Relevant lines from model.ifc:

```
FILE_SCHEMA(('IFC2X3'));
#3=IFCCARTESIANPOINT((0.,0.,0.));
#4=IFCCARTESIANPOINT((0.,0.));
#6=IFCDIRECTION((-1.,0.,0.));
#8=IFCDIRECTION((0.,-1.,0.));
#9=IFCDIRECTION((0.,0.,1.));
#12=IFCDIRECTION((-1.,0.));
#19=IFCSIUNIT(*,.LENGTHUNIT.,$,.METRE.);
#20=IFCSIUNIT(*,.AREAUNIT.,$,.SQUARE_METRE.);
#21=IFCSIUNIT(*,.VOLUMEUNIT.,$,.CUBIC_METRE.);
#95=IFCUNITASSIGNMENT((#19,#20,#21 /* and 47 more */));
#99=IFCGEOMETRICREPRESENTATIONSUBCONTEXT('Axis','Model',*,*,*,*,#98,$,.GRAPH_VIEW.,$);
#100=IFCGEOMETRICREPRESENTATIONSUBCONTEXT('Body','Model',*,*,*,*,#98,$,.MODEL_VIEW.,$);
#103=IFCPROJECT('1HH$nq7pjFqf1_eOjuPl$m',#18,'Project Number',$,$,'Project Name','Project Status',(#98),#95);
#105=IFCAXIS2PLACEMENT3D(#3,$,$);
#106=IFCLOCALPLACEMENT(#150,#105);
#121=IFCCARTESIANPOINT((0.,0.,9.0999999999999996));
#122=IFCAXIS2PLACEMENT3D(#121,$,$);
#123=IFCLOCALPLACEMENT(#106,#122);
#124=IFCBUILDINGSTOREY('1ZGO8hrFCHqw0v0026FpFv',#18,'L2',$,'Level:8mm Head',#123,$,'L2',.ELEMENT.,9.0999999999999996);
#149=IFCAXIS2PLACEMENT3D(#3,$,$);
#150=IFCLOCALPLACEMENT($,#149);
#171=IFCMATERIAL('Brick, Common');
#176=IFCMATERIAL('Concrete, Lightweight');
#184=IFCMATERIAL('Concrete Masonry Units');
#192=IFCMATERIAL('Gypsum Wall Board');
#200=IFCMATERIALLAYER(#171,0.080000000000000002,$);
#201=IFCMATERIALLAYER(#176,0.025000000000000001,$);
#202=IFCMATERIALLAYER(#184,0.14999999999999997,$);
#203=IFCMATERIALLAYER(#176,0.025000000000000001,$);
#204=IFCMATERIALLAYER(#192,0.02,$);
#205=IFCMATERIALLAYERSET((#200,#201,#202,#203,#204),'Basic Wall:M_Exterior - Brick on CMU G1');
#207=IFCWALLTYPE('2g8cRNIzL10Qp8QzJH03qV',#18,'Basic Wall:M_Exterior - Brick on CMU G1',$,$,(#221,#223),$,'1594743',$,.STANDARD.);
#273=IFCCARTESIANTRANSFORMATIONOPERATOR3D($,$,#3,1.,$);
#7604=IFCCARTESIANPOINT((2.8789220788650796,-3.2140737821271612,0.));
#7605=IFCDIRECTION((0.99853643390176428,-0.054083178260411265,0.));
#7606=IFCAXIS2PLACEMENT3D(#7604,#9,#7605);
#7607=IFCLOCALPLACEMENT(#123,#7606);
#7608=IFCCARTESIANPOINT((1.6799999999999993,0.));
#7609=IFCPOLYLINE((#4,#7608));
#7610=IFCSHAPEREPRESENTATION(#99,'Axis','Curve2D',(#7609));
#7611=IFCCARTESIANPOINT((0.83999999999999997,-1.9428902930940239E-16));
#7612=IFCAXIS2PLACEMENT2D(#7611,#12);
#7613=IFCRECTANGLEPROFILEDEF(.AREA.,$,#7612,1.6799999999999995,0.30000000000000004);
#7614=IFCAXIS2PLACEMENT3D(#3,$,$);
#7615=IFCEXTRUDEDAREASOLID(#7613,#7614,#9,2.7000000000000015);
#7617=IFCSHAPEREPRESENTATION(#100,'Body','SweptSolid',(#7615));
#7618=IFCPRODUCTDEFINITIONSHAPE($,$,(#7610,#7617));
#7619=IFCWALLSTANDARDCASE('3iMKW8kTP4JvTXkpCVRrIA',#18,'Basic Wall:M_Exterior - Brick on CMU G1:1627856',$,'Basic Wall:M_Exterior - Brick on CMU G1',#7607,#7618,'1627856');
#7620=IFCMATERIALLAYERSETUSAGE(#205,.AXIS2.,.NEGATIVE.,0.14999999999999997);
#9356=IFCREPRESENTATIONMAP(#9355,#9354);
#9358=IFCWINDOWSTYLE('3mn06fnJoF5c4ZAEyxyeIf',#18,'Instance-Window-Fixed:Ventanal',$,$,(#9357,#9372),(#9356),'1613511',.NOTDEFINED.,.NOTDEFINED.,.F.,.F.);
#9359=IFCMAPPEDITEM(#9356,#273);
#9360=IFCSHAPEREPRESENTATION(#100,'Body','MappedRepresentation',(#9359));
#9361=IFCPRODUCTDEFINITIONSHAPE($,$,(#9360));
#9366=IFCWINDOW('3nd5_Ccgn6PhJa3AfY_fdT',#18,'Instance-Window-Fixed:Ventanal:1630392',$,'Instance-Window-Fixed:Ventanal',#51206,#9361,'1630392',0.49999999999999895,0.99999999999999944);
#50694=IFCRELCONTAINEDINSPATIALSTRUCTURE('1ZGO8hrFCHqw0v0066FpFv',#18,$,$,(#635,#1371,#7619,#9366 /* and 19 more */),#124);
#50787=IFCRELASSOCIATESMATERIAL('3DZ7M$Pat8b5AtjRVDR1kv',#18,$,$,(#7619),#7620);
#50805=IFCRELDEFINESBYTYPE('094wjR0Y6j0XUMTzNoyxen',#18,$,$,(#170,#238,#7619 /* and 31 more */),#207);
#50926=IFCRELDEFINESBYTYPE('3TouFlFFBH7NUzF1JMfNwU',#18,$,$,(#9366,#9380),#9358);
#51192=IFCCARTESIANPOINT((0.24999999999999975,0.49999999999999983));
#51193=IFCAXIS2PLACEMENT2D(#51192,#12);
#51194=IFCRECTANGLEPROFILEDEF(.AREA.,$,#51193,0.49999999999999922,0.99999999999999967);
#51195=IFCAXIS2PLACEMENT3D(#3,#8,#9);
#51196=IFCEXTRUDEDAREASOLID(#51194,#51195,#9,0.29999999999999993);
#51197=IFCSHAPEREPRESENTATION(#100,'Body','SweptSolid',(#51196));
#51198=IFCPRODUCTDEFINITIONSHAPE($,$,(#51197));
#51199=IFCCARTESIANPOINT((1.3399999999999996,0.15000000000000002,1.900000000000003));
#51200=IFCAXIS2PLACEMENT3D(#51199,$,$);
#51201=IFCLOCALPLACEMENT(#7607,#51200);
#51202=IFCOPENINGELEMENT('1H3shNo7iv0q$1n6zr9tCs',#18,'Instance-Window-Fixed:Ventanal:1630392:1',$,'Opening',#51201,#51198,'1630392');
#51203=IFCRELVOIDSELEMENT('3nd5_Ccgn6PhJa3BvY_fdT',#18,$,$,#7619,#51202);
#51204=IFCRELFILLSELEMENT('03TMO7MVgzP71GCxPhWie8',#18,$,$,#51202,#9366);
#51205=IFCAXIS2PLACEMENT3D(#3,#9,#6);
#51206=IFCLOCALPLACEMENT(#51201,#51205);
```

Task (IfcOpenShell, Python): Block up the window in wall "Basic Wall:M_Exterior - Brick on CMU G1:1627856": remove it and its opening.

```python
import ifcopenshell
import ifcopenshell.api.feature
import ifcopenshell.api.root
import ifcopenshell.geom
import ifcopenshell.util.shape

model = ifcopenshell.open("model.ifc")
settings = ifcopenshell.geom.settings()


def volume(element):
    """Net volume in cubic metres, openings subtracted."""
    shape = ifcopenshell.geom.create_shape(settings, element)
    return ifcopenshell.util.shape.get_volume(shape.geometry)


window = model.by_id(9366)
opening = window.FillsVoids[0].RelatingOpeningElement
wall = opening.VoidsElements[0].RelatingBuildingElement
before = volume(wall)

ifcopenshell.api.root.remove_product(model, product=window)
ifcopenshell.api.feature.remove_feature(model, feature=opening)

after = volume(wall)

print(f"wall volume {before:.3f} -> {after:.3f} m3")

model.write("model_v2.ifc")
```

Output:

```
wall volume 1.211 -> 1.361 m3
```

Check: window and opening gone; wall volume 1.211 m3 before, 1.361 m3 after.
